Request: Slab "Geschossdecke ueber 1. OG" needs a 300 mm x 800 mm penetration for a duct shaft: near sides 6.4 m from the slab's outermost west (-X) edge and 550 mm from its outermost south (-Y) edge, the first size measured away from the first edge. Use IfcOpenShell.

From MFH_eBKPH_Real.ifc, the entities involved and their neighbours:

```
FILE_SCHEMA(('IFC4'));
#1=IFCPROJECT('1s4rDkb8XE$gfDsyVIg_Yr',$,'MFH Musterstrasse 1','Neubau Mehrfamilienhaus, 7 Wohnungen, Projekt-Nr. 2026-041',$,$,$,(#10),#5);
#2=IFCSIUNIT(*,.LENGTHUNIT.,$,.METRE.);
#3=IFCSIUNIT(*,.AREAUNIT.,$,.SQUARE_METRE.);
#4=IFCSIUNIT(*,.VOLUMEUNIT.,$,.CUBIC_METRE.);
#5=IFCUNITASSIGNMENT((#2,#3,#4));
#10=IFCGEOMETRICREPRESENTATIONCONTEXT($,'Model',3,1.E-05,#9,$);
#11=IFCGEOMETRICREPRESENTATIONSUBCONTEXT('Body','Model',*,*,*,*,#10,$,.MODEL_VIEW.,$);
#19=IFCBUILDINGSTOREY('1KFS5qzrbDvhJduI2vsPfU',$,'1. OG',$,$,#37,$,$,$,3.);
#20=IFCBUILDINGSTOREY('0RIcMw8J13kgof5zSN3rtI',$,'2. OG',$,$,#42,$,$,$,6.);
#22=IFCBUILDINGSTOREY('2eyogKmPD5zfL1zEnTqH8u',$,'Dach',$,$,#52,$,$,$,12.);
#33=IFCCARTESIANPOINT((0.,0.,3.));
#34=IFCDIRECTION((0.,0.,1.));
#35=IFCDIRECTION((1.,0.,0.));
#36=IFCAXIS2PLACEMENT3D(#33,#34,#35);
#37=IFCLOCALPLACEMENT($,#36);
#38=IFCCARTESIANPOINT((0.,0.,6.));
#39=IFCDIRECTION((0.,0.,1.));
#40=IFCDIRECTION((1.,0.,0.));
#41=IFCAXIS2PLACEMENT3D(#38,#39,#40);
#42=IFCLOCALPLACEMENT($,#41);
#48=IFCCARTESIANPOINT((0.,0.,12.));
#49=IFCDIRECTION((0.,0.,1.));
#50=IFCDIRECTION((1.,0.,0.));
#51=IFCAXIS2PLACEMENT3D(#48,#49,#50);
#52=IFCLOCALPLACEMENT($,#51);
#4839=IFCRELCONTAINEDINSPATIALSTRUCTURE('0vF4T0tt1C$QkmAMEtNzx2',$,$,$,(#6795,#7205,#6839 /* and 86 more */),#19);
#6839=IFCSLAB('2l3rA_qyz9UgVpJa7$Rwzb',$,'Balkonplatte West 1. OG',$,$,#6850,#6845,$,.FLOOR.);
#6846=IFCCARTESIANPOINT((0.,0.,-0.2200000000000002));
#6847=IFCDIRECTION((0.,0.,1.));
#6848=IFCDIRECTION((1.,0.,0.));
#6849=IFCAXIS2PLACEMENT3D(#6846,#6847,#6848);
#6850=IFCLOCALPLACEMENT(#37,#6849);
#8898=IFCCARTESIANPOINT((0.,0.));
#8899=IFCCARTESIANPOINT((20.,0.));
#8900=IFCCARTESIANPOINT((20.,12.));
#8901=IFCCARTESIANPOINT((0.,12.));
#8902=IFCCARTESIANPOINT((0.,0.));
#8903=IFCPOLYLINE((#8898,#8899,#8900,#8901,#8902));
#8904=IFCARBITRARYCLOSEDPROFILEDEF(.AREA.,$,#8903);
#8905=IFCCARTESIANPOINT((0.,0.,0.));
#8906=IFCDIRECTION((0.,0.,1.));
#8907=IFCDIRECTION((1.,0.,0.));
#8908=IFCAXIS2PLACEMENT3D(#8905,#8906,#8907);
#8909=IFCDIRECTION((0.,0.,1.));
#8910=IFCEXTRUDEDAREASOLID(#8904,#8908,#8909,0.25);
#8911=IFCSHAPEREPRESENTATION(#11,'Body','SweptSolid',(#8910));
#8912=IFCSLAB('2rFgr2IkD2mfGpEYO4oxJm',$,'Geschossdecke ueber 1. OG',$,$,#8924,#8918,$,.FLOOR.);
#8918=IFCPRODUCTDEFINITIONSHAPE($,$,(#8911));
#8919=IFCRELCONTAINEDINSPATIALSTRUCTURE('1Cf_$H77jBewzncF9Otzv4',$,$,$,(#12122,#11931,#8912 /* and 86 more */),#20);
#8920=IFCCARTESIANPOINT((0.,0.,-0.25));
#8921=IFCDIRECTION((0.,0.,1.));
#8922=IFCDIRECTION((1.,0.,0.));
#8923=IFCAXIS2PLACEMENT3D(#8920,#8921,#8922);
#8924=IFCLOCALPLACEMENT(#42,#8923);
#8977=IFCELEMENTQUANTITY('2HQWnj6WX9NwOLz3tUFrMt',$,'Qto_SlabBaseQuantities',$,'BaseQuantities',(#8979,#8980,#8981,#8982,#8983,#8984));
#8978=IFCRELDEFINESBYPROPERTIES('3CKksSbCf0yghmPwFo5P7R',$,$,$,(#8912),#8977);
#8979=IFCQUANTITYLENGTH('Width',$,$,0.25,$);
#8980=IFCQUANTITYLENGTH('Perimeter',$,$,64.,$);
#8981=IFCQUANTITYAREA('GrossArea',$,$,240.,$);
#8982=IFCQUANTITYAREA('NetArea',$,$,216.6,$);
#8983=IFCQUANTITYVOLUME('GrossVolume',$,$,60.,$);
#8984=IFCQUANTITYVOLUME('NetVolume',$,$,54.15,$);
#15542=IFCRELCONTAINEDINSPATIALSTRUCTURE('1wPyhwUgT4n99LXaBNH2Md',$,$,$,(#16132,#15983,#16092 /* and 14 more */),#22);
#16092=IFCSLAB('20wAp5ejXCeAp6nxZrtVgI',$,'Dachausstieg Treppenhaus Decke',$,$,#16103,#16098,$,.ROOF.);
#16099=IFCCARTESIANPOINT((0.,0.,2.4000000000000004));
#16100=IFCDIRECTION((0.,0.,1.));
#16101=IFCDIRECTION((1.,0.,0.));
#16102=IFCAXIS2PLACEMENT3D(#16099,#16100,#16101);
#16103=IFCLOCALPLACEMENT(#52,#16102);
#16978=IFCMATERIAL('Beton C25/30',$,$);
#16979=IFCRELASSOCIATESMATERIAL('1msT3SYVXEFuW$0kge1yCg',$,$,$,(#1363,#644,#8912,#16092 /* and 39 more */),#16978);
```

```python
import numpy as np
import ifcopenshell
import ifcopenshell.api.feature
import ifcopenshell.api.geometry
import ifcopenshell.api.pset
import ifcopenshell.api.root
import ifcopenshell.geom
import ifcopenshell.util.element
import ifcopenshell.util.placement
import ifcopenshell.util.representation
import ifcopenshell.util.shape
import ifcopenshell.util.unit

model = ifcopenshell.open("MFH_eBKPH_Real.ifc")
unit_scale = ifcopenshell.util.unit.calculate_unit_scale(model)
area_scale = ifcopenshell.util.unit.calculate_unit_scale(model, "AREAUNIT")
volume_scale = ifcopenshell.util.unit.calculate_unit_scale(model, "VOLUMEUNIT")
settings = ifcopenshell.geom.settings()


def volume(element):
    """Net volume in cubic metres, openings subtracted."""
    shape = ifcopenshell.geom.create_shape(settings, element)
    return ifcopenshell.util.shape.get_volume(shape.geometry)


slab = model.by_guid("2rFgr2IkD2mfGpEYO4oxJm")
before = volume(slab)

# Extent in the slab's own axes, in metres. The edges named are its -X and -Y sides.
slab_shape = ifcopenshell.geom.create_shape(settings, slab)
vertices = ifcopenshell.util.shape.get_vertices(slab_shape.geometry)
x_min, y_min, bottom = vertices.min(axis=0)
top = vertices[:, 2].max()

opening = ifcopenshell.api.root.create_entity(model, ifc_class="IfcOpeningElement", name="Duct shaft opening", predefined_type="OPENING")
context = ifcopenshell.util.representation.get_context(model, "Model", "Body", "MODEL_VIEW")
width, depth = 0.3, 0.8
outline = [(0.0, 0.0), (width, 0.0), (width, depth), (0.0, depth), (0.0, 0.0)]
# Overshoot both faces by 50 mm so the cut is clean.
shape = ifcopenshell.api.geometry.add_slab_representation(
    model, context=context, depth=top - bottom + 0.1, polyline=outline
)
ifcopenshell.api.geometry.assign_representation(model, product=opening, representation=shape)

matrix = ifcopenshell.util.placement.get_local_placement(slab.ObjectPlacement)
matrix[:, 3] = matrix @ np.append(np.array([x_min + 6.4, y_min + 0.55, bottom - 0.05]) / unit_scale, 1.0)
ifcopenshell.api.geometry.edit_object_placement(model, product=opening, matrix=matrix, is_si=False)
ifcopenshell.api.feature.add_feature(model, feature=opening, element=slab)

after = volume(slab)

# Update the slab's stored quantities.
qto = model.by_id(ifcopenshell.util.element.get_pset(slab, "Qto_SlabBaseQuantities", should_inherit=False)["id"])
ifcopenshell.api.pset.edit_qto(model, qto=qto, properties={
    "NetArea": after / (top - bottom) / area_scale,
    "NetVolume": after / volume_scale,
})

print(f"slab volume {before:.3f} -> {after:.3f} m3")

model.write("MFH_eBKPH_Real_rev.ifc")
```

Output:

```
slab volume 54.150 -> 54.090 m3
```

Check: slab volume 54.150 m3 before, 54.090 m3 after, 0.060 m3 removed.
